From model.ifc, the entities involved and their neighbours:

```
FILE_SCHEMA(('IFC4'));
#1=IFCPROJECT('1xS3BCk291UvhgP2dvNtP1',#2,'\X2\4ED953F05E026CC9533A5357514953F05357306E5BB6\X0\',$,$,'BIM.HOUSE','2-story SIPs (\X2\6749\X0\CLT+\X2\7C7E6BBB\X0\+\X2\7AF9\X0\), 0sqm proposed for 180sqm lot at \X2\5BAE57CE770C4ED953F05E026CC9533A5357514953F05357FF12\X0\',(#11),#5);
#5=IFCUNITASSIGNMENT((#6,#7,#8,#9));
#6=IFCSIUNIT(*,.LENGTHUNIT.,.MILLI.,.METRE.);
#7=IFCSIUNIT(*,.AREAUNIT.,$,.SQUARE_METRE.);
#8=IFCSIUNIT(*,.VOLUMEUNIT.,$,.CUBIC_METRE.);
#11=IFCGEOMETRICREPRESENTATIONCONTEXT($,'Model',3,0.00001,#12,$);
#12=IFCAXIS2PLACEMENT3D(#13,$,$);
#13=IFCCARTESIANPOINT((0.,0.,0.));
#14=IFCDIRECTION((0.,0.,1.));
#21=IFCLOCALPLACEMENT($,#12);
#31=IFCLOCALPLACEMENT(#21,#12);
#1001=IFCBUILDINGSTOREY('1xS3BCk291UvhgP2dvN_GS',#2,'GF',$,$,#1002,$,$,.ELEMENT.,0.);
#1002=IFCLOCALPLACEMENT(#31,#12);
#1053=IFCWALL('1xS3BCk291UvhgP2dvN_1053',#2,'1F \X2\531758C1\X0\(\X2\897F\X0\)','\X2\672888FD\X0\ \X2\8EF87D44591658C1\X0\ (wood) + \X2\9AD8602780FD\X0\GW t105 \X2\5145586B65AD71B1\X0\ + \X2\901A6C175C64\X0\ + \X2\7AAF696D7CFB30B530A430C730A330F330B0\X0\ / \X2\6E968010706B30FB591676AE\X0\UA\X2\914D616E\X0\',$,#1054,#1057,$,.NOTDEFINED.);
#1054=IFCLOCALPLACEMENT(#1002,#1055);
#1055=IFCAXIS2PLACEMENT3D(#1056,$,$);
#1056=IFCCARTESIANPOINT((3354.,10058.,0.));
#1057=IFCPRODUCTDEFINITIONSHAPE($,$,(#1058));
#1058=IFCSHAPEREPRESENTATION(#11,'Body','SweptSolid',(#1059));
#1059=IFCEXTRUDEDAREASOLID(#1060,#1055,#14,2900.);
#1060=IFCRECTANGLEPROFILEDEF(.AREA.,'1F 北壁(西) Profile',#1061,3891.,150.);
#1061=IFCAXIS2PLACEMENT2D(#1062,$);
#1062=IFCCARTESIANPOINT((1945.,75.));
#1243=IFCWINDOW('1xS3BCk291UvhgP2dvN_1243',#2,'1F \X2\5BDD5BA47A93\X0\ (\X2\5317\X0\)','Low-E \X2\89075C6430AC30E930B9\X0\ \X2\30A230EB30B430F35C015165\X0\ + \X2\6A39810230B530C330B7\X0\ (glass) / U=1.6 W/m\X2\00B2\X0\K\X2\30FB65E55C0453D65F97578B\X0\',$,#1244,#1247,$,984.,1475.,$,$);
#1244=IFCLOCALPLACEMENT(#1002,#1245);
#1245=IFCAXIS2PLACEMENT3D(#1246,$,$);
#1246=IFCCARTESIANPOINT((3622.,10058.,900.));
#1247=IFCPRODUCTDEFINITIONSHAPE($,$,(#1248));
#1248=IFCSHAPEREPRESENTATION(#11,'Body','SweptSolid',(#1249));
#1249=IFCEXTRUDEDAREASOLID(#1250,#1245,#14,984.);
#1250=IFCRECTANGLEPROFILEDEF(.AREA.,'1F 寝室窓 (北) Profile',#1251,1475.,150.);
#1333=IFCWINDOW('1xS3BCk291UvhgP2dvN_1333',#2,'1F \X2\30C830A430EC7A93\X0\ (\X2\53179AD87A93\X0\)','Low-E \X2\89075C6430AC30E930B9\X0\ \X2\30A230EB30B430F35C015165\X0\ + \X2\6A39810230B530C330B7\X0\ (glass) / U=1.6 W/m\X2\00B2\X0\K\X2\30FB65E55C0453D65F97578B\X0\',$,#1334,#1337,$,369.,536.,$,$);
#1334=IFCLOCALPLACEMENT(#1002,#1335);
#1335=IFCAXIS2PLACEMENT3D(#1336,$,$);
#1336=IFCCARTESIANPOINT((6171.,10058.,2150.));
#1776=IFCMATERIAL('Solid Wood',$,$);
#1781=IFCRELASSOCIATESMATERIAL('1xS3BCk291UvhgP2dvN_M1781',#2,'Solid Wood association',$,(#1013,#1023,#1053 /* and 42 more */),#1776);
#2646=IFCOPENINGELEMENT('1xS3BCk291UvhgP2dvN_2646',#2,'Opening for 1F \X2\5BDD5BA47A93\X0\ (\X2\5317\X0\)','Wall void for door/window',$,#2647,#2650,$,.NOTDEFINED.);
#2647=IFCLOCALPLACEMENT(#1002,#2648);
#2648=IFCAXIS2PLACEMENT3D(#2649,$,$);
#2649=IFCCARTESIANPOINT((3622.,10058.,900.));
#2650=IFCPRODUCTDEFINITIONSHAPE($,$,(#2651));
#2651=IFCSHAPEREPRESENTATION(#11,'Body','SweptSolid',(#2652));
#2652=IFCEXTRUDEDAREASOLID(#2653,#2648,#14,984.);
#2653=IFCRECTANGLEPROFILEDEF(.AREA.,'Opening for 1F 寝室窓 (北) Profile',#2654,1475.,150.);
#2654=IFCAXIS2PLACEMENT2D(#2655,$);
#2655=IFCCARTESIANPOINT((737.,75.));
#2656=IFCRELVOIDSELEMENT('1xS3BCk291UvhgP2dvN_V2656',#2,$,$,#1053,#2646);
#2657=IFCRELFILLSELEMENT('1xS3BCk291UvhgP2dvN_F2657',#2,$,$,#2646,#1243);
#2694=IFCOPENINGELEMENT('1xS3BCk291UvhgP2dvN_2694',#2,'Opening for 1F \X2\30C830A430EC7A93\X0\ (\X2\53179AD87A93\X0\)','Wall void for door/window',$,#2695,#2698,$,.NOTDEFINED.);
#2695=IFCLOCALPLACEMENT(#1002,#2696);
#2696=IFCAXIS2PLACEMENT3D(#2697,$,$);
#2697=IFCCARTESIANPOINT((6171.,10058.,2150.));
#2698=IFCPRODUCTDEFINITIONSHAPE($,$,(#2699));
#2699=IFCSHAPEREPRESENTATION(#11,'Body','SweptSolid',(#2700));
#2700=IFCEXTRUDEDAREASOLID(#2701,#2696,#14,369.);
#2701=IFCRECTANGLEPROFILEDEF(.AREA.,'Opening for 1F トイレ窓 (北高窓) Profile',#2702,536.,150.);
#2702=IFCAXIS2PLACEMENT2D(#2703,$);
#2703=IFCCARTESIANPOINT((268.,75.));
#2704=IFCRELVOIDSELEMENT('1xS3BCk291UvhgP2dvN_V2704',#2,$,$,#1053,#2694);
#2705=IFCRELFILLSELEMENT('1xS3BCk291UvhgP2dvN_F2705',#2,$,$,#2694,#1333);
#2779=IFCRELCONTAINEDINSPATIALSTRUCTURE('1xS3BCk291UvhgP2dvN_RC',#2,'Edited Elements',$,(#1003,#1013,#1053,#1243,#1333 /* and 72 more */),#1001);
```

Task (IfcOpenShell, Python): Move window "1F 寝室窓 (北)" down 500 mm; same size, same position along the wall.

```python
import numpy as np
import ifcopenshell
import ifcopenshell.api.geometry
import ifcopenshell.util.placement
import ifcopenshell.util.unit

model = ifcopenshell.open("model.ifc")
unit_scale = ifcopenshell.util.unit.calculate_unit_scale(model)

window = model.by_id(1243)
opening = window.FillsVoids[0].RelatingOpeningElement
dz = -0.5 / unit_scale

shift = np.array([0.0, 0.0, dz])
# The window is not placed relative to its opening, so move both.
for product in (opening, window):
    matrix = ifcopenshell.util.placement.get_local_placement(product.ObjectPlacement)
    matrix[:3, 3] += shift
    ifcopenshell.api.geometry.edit_object_placement(model, product=product, matrix=matrix, is_si=False)

print(f"moved by {dz * unit_scale:+.3f} m")

model.write("model_edited.ifc")
```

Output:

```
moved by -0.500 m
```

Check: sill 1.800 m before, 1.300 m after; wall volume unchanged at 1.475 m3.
